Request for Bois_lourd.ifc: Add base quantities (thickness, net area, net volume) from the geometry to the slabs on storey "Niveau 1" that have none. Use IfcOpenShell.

First a look at what the model holds.

```python
import ifcopenshell
import ifcopenshell.util.element
import ifcopenshell.util.unit

model = ifcopenshell.open("Bois_lourd.ifc")
print(model.schema)
for unit_type in ("LENGTHUNIT", "AREAUNIT", "VOLUMEUNIT"):
    print(unit_type, ifcopenshell.util.unit.calculate_unit_scale(model, unit_type))
storey = next(s for s in model.by_type("IfcBuildingStorey") if s.Name == "Niveau 1")
slabs = [e for e in ifcopenshell.util.element.get_decomposition(storey) if e.is_a("IfcSlab")]
for e in sorted(slabs, key=lambda e: e.id()):
    print(e.id(), e.is_a(), e.Name, list(ifcopenshell.util.element.get_psets(e, qtos_only=True)), sep=" | ")
```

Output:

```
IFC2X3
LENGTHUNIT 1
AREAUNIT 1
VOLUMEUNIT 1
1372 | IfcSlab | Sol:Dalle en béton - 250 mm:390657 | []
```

```python
import ifcopenshell
import ifcopenshell.api.pset
import ifcopenshell.geom
import ifcopenshell.util.element
import ifcopenshell.util.shape
import ifcopenshell.util.unit

model = ifcopenshell.open("Bois_lourd.ifc")
unit_scale = ifcopenshell.util.unit.calculate_unit_scale(model)
area_scale = ifcopenshell.util.unit.calculate_unit_scale(model, "AREAUNIT")
volume_scale = ifcopenshell.util.unit.calculate_unit_scale(model, "VOLUMEUNIT")
settings = ifcopenshell.geom.settings()

storey = next(s for s in model.by_type("IfcBuildingStorey") if s.Name == "Niveau 1")
slabs = [e for e in ifcopenshell.util.element.get_decomposition(storey) if e.is_a("IfcSlab")]

for e in sorted(slabs, key=lambda e: e.id()):
    if ifcopenshell.util.element.get_psets(e, qtos_only=True, should_inherit=False):
        continue
    # Geometry comes back in metres, in the element's own axes.
    shape = ifcopenshell.geom.create_shape(settings, e)
    values = {
        "Width": ifcopenshell.util.shape.get_z(shape.geometry) / unit_scale,
        "NetArea": ifcopenshell.util.shape.get_footprint_area(shape.geometry) / area_scale,
        "NetVolume": ifcopenshell.util.shape.get_volume(shape.geometry) / volume_scale,
    }
    qto = ifcopenshell.api.pset.add_qto(model, product=e, name="BaseQuantities")
    ifcopenshell.api.pset.edit_qto(model, qto=qto, properties=values)
    print(e.id(), {k: round(v, 3) for k, v in values.items()})

model.write("Bois_lourd_updated.ifc")
```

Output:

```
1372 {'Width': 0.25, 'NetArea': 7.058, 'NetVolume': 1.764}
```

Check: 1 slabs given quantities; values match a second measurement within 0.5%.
